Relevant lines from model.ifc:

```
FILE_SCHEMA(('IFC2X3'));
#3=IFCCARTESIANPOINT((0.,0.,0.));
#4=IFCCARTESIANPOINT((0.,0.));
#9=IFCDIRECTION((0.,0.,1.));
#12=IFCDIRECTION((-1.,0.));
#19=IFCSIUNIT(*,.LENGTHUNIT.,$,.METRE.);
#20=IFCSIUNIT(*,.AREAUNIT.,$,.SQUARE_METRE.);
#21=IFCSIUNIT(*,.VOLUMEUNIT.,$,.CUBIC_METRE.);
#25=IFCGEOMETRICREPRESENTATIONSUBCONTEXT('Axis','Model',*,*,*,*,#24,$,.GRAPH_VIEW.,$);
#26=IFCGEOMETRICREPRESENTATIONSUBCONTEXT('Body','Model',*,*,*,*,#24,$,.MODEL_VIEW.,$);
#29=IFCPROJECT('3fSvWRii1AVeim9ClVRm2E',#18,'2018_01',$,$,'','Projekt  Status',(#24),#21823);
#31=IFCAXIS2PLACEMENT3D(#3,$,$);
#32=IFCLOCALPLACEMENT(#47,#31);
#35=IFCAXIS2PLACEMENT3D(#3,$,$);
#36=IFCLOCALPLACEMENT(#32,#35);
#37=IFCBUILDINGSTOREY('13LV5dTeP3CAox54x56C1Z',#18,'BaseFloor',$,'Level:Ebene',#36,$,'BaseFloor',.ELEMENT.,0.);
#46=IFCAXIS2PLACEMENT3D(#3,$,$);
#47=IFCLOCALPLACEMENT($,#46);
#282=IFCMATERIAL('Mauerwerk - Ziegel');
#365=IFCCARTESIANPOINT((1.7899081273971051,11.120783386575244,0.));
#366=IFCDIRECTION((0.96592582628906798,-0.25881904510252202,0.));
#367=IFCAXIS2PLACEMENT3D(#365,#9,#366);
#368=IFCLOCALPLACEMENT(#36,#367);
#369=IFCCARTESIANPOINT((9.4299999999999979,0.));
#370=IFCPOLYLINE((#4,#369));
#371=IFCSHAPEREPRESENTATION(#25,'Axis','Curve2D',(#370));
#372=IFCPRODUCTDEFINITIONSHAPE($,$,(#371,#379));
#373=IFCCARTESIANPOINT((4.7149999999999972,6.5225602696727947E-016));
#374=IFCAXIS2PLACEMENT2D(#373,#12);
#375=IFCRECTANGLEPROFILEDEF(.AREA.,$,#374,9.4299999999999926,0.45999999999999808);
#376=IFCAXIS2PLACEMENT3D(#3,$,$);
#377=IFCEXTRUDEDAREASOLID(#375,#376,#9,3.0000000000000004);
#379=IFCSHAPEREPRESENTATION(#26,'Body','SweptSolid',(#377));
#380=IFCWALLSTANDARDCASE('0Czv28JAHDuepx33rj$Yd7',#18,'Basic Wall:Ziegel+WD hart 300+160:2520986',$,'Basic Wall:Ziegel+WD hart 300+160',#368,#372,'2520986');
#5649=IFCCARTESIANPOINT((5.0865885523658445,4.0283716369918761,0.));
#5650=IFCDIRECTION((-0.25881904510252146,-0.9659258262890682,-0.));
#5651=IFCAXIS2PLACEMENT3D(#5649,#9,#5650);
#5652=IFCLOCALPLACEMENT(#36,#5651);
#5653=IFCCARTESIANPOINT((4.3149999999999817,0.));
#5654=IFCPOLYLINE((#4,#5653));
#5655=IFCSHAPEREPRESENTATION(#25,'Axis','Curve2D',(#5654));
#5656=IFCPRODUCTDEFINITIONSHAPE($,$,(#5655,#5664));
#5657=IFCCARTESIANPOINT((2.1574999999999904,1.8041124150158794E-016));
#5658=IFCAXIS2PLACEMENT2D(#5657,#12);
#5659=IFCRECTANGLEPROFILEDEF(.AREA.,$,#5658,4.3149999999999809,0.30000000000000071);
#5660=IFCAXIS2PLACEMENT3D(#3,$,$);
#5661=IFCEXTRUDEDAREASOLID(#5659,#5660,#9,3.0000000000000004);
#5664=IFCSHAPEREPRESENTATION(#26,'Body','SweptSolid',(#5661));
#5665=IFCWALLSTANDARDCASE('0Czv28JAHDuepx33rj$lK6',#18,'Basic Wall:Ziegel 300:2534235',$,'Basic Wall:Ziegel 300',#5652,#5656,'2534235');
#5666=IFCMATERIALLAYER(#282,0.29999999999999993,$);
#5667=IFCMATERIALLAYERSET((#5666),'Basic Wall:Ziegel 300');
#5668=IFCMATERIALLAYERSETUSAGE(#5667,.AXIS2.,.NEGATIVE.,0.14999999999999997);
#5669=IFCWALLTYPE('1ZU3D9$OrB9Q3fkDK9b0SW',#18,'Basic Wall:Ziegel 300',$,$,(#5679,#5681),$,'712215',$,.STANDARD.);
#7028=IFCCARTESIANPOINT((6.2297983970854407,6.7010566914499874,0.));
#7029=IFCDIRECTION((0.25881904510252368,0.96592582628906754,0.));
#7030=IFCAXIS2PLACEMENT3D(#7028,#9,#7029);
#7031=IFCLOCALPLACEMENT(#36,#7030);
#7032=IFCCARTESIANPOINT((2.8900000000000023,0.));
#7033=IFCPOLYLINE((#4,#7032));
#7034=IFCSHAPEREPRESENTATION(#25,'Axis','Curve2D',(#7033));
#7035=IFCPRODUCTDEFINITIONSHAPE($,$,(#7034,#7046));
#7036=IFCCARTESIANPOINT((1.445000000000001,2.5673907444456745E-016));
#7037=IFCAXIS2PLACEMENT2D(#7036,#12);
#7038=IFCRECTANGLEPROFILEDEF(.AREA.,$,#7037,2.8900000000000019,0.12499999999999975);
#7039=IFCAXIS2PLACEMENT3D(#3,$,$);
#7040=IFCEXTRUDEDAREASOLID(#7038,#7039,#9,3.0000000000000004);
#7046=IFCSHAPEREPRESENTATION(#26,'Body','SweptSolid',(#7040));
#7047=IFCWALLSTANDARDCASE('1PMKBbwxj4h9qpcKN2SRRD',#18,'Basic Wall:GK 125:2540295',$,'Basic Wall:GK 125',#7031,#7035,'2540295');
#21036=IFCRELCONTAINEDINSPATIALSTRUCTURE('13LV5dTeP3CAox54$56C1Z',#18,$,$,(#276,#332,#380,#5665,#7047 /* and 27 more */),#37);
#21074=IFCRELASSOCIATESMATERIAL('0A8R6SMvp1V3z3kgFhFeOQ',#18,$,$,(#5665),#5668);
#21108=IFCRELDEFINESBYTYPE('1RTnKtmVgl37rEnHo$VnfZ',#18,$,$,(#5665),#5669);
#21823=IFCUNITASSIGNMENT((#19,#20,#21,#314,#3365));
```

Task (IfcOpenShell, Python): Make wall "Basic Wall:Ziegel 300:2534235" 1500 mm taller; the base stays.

```python
import ifcopenshell
import ifcopenshell.geom
import ifcopenshell.util.representation
import ifcopenshell.util.shape

model = ifcopenshell.open("model.ifc")
settings = ifcopenshell.geom.settings()


def volume(element):
    """Net volume in cubic metres, openings subtracted."""
    shape = ifcopenshell.geom.create_shape(settings, element)
    return ifcopenshell.util.shape.get_volume(shape.geometry)


wall = model.by_guid("0Czv28JAHDuepx33rj$lK6")
before = volume(wall)

body = ifcopenshell.util.representation.get_representation(wall, "Model", "Body")
solid = body.Items[0]
old_height = solid.Depth
solid.Depth += 1.5
after = volume(wall)

print(f"height {old_height:g} -> {solid.Depth:g}, volume {before:.3f} -> {after:.3f} m3")

model.write("model_rev.ifc")
```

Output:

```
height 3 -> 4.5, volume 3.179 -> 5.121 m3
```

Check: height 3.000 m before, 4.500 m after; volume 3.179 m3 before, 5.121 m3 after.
